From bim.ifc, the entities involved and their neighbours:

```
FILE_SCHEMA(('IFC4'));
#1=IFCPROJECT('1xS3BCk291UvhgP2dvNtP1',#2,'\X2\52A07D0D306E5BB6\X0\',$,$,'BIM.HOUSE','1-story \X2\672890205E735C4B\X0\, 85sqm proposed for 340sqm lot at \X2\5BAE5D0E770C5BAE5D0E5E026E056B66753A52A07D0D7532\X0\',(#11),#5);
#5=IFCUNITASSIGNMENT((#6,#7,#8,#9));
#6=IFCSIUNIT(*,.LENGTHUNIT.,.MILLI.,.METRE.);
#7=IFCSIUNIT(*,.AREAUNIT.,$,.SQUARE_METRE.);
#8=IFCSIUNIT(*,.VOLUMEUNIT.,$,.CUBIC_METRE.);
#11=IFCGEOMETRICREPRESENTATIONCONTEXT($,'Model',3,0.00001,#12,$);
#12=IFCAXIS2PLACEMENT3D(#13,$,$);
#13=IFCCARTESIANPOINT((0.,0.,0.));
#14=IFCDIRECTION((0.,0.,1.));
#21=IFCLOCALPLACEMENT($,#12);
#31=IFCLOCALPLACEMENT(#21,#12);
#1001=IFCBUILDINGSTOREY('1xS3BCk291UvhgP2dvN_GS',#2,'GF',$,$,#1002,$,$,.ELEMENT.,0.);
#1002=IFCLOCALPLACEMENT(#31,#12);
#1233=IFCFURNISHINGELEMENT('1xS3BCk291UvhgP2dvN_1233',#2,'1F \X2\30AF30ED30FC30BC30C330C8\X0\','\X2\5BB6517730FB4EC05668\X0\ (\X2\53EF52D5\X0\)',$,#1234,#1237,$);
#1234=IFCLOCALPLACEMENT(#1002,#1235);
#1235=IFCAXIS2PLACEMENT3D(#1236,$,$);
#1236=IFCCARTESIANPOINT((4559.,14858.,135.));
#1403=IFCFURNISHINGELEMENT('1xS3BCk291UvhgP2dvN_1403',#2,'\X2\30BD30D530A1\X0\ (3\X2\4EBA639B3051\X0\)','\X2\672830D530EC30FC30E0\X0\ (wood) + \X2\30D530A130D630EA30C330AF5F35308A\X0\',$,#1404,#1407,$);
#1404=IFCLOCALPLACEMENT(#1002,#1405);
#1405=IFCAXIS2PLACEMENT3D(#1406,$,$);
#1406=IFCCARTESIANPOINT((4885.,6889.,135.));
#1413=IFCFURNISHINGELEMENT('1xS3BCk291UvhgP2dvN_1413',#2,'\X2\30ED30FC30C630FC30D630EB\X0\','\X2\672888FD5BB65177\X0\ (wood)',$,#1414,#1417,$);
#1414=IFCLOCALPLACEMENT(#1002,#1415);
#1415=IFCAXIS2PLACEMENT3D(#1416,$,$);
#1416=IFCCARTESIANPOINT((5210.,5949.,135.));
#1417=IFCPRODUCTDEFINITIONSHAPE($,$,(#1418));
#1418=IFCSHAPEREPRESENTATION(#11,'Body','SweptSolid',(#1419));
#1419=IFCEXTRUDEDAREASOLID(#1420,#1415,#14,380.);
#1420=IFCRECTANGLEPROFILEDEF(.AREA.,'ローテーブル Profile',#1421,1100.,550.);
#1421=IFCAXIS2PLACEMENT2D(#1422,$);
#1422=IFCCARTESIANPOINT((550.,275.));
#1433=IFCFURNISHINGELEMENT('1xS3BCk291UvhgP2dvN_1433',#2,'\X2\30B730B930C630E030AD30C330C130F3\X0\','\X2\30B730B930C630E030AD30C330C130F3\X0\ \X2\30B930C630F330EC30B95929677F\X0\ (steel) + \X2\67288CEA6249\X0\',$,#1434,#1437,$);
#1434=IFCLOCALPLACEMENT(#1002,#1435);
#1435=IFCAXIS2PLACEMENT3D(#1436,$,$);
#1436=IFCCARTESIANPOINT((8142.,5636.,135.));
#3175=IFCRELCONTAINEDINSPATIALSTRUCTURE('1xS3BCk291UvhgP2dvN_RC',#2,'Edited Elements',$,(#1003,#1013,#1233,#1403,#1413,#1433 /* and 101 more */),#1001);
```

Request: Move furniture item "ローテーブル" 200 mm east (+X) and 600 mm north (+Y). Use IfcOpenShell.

```python
import ifcopenshell
import ifcopenshell.api.geometry
import ifcopenshell.util.placement

model = ifcopenshell.open("bim.ifc")

item = model.by_guid("1xS3BCk291UvhgP2dvN_1413")
matrix = ifcopenshell.util.placement.get_local_placement(item.ObjectPlacement)
matrix[0, 3] += 200.0
matrix[1, 3] += 600.0
ifcopenshell.api.geometry.edit_object_placement(model, product=item, matrix=matrix, is_si=False)

print(ifcopenshell.util.placement.get_local_placement(item.ObjectPlacement).round(3) + 0.0)

model.write("bim_v2.ifc")
```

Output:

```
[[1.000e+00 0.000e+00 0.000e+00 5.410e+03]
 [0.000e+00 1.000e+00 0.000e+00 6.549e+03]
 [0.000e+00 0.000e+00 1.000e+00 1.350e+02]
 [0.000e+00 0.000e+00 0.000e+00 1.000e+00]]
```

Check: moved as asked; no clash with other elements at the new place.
